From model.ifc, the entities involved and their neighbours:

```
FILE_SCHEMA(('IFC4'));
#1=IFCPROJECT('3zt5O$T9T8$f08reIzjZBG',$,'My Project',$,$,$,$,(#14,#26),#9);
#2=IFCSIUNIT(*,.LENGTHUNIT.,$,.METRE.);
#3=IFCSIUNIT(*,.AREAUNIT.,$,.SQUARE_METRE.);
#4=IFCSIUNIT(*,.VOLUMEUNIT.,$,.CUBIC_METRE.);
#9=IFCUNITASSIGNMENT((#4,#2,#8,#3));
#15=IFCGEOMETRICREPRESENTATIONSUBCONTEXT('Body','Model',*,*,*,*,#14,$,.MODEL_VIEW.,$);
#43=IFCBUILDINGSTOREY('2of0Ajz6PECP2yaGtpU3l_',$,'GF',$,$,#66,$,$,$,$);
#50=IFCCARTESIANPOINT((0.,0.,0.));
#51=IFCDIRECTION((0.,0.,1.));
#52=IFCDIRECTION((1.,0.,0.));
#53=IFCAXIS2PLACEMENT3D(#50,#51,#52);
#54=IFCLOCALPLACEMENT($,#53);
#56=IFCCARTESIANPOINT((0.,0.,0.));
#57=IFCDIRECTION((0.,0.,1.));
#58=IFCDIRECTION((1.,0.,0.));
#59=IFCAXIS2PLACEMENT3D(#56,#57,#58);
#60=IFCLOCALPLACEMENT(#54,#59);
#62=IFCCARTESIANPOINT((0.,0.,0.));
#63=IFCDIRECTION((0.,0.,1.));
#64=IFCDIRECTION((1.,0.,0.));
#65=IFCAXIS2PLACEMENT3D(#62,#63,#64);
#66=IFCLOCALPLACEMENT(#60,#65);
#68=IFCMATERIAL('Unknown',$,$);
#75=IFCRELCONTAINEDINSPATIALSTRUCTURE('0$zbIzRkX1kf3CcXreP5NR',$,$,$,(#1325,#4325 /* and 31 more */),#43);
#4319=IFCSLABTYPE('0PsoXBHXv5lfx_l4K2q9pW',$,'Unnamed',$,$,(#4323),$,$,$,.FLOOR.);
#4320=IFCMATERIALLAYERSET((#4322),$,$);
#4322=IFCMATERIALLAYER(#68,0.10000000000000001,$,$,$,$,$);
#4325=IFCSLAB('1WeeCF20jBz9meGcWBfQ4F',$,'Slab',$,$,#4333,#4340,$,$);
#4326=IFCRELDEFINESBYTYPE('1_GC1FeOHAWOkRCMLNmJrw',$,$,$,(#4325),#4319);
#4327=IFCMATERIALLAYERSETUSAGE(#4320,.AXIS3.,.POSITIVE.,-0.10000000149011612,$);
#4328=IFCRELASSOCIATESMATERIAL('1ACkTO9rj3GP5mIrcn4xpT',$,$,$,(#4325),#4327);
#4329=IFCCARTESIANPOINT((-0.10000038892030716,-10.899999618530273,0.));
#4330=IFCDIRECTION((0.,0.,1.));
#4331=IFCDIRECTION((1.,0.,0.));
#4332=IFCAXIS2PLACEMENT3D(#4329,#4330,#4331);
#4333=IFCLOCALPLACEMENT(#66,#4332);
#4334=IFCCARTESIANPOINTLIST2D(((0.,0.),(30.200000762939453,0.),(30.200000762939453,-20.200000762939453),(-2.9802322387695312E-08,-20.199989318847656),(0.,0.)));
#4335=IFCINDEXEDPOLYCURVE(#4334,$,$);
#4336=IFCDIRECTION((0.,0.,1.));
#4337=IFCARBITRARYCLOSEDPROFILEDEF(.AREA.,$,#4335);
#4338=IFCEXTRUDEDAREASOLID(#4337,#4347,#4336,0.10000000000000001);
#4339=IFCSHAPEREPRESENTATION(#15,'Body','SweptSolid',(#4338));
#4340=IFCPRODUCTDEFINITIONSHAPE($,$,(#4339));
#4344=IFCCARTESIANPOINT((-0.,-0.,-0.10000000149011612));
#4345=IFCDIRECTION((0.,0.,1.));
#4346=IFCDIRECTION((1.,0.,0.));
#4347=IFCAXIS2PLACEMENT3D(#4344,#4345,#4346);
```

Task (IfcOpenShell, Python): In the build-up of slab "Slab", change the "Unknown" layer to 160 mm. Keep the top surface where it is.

```python
import ifcopenshell
import ifcopenshell.util.element
import ifcopenshell.util.representation

model = ifcopenshell.open("model.ifc")

layer_set = model.by_id(4320)
layer = next(l for l in layer_set.MaterialLayers if l.Material and l.Material.Name == "Unknown")
change = 0.16 - layer.LayerThickness
layer.LayerThickness += change

# Geometry does not follow the layer set by itself.
slabs = [e for e in ifcopenshell.util.element.get_elements_by_material(model, layer_set) if e.is_a("IfcSlab")]
for slab in sorted(slabs, key=lambda e: e.id()):
    body = ifcopenshell.util.representation.get_representation(slab, "Model", "Body")
    solid = body.Items[0]
    old_depth = solid.Depth
    solid.Depth += change
    # Extruded upwards: lower the start of the extrusion so the top stays.
    x, y, z = solid.Position.Location.Coordinates
    solid.Position.Location = model.createIfcCartesianPoint((x, y, z - change))
    print(slab.id(), f"{old_depth:g} -> {solid.Depth:g}")

# The layers are counted up from the underside, which has moved.
for usage in {ifcopenshell.util.element.get_material(slab) for slab in slabs}:
    usage.OffsetFromReferenceLine -= change

model.write("model_rev.ifc")
```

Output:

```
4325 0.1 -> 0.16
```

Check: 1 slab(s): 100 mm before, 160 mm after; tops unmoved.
